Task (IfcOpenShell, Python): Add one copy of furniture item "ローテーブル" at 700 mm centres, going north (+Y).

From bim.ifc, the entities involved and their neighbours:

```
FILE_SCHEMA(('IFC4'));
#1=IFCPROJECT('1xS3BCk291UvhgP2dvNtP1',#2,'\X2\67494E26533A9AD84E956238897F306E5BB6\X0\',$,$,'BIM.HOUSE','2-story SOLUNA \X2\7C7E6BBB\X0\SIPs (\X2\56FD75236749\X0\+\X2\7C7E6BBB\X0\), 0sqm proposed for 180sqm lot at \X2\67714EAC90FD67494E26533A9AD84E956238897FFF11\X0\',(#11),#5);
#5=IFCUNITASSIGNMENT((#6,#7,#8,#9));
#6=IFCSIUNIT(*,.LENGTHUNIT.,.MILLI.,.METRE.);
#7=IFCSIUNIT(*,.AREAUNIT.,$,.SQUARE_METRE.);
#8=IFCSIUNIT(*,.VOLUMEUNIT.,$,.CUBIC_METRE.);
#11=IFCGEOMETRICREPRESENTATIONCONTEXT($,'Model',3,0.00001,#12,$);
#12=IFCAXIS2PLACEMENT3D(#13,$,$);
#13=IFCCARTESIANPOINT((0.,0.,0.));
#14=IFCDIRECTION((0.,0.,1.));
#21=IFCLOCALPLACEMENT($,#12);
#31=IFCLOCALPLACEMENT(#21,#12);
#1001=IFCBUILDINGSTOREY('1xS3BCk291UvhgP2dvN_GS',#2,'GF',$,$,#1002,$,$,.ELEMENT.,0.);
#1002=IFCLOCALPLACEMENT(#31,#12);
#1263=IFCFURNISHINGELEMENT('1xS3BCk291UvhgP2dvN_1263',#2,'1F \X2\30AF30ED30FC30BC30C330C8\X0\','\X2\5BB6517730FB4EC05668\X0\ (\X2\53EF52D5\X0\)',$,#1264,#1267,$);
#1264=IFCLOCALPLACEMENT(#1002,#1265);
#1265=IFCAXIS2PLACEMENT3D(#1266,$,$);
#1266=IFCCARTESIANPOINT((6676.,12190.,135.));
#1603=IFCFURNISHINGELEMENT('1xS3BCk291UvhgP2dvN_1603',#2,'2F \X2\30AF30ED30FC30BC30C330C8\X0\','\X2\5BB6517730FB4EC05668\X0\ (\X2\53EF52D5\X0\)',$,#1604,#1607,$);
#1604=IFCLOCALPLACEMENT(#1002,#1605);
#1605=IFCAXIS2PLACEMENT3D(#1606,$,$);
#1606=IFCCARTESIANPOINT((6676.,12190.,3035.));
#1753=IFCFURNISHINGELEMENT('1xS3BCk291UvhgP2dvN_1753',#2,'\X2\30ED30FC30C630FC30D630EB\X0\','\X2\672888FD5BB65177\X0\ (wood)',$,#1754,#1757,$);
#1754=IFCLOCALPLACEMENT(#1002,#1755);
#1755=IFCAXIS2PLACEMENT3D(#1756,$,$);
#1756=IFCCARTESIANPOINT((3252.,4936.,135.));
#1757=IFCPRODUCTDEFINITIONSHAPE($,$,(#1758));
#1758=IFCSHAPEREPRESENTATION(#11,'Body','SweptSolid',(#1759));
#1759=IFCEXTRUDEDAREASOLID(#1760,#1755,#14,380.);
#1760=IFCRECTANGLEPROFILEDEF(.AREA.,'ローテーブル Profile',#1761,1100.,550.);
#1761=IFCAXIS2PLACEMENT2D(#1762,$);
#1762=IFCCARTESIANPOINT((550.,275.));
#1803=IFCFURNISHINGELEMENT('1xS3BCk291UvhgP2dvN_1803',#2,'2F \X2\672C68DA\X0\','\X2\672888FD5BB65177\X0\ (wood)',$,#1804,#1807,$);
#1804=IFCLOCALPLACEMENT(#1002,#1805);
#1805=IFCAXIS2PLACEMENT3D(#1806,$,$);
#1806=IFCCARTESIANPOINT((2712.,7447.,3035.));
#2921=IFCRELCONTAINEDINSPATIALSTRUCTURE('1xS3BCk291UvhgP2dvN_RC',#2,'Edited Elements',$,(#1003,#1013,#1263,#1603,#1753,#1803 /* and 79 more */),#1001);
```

```python
import numpy as np
import ifcopenshell
import ifcopenshell.api.geometry
import ifcopenshell.api.root
import ifcopenshell.util.element
import ifcopenshell.util.placement
import ifcopenshell.util.unit

model = ifcopenshell.open("bim.ifc")
unit_scale = ifcopenshell.util.unit.calculate_unit_scale(model)


def reuse_history(source, copy):
    """copy_class also copies each property set's owner history, people and application; keep the originals."""
    for rel in copy.IsDefinedBy:
        if rel.is_a("IfcRelDefinesByProperties") and (history := rel.RelatingPropertyDefinition.OwnerHistory):
            rel.RelatingPropertyDefinition.OwnerHistory = source.OwnerHistory
            ifcopenshell.util.element.remove_deep2(model, history)


source = model.by_guid("1xS3BCk291UvhgP2dvN_1753")
base = ifcopenshell.util.placement.get_local_placement(source.ObjectPlacement)
step = np.array([0.0, 1.0, 0.0]) * 0.7 / unit_scale

for i in range(1, 2):
    copy = ifcopenshell.api.root.copy_class(model, product=source)
    copy.Representation = ifcopenshell.util.element.copy_deep(
        model, source.Representation, exclude=["IfcGeometricRepresentationContext", "IfcRepresentationMap"]
    )
    reuse_history(source, copy)
    matrix = base.copy()
    matrix[:3, 3] += i * step
    print("added at", matrix[:3, 3].round(3) + 0.0)
    ifcopenshell.api.geometry.edit_object_placement(model, product=copy, matrix=matrix, is_si=False)

model.write("bim_updated.ifc")
```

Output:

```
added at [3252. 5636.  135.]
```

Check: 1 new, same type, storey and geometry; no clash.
